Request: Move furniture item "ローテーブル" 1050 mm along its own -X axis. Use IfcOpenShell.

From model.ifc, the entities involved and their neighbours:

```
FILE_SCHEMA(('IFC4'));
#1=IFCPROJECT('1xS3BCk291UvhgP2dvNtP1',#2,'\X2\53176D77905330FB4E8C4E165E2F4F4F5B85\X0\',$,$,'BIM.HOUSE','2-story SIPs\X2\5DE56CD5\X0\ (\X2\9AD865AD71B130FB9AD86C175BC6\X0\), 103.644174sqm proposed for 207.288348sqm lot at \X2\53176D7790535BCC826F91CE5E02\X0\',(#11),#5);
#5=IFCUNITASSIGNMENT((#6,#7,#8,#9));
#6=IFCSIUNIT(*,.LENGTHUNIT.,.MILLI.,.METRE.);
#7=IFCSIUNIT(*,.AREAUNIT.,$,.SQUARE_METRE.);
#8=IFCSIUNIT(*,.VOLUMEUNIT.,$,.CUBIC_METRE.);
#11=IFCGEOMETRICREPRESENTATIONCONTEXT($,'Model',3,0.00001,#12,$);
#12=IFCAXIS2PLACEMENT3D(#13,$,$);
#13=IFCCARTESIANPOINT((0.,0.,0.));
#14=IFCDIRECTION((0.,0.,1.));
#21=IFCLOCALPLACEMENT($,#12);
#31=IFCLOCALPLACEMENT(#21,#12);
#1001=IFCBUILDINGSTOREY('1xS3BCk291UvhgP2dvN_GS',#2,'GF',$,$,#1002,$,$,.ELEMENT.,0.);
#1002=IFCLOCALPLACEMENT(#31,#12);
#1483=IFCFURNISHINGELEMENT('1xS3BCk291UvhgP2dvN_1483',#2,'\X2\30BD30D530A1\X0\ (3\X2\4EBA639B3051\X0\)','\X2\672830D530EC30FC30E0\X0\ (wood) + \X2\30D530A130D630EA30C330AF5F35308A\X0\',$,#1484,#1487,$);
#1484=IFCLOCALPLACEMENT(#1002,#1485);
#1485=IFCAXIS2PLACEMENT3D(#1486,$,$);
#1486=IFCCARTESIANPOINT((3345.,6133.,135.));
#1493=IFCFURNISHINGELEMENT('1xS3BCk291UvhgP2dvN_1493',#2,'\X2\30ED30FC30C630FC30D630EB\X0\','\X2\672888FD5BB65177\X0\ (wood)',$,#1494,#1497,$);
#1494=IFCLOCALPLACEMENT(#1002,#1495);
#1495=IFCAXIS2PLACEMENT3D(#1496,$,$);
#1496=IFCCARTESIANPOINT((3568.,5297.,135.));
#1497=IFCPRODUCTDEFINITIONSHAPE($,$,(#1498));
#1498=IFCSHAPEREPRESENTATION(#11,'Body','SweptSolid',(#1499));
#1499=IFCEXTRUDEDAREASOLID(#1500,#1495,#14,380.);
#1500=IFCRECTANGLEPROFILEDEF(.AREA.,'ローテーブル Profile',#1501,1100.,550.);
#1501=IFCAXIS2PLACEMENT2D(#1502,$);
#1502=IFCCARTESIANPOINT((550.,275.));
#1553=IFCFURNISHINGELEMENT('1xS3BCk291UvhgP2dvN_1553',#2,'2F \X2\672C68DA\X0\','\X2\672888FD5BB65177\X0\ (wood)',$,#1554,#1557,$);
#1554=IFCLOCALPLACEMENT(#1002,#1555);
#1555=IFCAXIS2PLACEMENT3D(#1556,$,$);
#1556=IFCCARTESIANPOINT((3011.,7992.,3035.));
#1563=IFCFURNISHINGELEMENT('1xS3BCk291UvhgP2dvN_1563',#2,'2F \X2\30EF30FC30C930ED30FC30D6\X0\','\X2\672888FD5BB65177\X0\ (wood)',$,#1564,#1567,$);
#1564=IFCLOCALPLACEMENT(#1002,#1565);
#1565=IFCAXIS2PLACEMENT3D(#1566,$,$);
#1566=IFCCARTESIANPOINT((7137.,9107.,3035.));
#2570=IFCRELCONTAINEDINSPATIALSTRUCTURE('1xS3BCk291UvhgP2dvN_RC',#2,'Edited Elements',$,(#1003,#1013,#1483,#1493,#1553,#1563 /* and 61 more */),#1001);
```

```python
import ifcopenshell
import ifcopenshell.api.geometry
import ifcopenshell.util.placement

model = ifcopenshell.open("model.ifc")

item = model.by_guid("1xS3BCk291UvhgP2dvN_1493")
matrix = ifcopenshell.util.placement.get_local_placement(item.ObjectPlacement)
matrix[:3, 3] -= matrix[:3, 0] * 1050.0
ifcopenshell.api.geometry.edit_object_placement(model, product=item, matrix=matrix, is_si=False)

print(ifcopenshell.util.placement.get_local_placement(item.ObjectPlacement).round(3) + 0.0)

model.write("model-out.ifc")
```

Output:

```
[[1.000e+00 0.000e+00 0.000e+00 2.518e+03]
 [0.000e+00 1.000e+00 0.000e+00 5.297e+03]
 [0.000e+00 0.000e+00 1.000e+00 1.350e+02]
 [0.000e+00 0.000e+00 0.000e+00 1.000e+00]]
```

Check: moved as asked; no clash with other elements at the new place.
